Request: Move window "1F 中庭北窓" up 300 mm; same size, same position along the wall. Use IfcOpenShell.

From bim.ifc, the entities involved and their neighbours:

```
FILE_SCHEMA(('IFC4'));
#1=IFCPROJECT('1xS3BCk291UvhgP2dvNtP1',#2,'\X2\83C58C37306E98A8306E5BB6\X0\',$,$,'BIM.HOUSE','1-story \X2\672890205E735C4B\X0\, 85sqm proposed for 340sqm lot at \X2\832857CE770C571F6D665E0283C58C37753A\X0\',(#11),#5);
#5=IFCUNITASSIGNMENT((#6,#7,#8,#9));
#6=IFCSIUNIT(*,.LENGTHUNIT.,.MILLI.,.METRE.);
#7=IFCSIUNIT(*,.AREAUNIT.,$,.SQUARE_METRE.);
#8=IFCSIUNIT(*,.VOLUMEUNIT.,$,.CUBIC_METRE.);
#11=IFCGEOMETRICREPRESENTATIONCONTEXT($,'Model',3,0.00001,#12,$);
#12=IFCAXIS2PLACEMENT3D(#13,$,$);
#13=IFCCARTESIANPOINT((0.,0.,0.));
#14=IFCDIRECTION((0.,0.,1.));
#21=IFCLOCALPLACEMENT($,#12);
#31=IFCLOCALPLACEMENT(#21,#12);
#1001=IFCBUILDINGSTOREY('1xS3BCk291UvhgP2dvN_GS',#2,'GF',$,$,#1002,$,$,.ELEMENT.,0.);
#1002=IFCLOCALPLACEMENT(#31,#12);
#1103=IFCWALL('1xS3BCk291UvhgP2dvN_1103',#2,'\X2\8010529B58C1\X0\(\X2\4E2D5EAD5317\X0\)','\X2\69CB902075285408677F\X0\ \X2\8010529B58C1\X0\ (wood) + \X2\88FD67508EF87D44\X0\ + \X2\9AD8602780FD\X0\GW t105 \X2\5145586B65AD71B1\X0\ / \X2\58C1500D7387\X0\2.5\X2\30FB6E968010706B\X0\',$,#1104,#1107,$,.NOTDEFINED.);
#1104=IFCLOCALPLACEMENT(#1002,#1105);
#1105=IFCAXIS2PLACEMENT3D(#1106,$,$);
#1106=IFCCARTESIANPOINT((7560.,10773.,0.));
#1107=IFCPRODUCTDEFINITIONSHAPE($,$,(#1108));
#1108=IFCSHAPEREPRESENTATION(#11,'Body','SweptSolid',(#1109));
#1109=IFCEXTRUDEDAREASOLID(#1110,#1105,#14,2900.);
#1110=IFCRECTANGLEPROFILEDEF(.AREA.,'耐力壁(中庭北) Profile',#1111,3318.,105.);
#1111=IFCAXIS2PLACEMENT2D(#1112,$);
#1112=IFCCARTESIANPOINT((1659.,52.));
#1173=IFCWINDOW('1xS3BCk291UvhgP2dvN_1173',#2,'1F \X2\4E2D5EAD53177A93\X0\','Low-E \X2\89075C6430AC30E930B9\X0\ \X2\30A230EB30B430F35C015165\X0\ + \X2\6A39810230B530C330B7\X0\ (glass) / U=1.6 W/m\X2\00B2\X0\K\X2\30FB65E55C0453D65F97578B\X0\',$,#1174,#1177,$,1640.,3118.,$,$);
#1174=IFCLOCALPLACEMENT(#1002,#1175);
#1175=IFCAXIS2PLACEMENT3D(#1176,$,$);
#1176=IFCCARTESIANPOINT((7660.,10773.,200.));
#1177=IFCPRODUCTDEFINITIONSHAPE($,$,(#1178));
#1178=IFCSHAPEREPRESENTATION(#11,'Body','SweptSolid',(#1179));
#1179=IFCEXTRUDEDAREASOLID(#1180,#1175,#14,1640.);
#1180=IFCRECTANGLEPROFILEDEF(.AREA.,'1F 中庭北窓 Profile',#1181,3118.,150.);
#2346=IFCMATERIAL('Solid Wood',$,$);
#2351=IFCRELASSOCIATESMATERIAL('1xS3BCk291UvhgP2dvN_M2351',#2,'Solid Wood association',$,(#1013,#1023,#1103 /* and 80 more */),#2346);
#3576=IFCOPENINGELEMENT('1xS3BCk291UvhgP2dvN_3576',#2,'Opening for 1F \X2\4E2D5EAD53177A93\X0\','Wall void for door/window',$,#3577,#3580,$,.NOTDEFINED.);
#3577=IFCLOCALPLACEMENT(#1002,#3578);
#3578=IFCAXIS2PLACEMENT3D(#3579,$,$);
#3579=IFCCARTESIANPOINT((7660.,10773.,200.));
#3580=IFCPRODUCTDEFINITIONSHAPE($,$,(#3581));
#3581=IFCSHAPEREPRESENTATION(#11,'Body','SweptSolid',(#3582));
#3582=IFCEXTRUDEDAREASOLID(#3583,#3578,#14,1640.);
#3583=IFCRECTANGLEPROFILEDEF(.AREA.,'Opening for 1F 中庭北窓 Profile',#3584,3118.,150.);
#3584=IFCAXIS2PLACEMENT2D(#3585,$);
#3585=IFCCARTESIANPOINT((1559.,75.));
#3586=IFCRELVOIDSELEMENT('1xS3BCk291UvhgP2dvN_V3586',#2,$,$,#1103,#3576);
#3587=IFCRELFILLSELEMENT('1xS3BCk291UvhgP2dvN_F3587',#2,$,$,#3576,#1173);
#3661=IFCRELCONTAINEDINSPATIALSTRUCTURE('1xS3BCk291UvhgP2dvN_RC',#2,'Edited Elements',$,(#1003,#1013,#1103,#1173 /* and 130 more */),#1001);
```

```python
import numpy as np
import ifcopenshell
import ifcopenshell.api.geometry
import ifcopenshell.util.placement
import ifcopenshell.util.unit

model = ifcopenshell.open("bim.ifc")
unit_scale = ifcopenshell.util.unit.calculate_unit_scale(model)

window = model.by_id(1173)
opening = window.FillsVoids[0].RelatingOpeningElement
dz = 0.3 / unit_scale

shift = np.array([0.0, 0.0, dz])
# The window is not placed relative to its opening, so move both.
for product in (opening, window):
    matrix = ifcopenshell.util.placement.get_local_placement(product.ObjectPlacement)
    matrix[:3, 3] += shift
    ifcopenshell.api.geometry.edit_object_placement(model, product=product, matrix=matrix, is_si=False)

print(f"moved by {dz * unit_scale:+.3f} m")

model.write("bim_updated.ifc")
```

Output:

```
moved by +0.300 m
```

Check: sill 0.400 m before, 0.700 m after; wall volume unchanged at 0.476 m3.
